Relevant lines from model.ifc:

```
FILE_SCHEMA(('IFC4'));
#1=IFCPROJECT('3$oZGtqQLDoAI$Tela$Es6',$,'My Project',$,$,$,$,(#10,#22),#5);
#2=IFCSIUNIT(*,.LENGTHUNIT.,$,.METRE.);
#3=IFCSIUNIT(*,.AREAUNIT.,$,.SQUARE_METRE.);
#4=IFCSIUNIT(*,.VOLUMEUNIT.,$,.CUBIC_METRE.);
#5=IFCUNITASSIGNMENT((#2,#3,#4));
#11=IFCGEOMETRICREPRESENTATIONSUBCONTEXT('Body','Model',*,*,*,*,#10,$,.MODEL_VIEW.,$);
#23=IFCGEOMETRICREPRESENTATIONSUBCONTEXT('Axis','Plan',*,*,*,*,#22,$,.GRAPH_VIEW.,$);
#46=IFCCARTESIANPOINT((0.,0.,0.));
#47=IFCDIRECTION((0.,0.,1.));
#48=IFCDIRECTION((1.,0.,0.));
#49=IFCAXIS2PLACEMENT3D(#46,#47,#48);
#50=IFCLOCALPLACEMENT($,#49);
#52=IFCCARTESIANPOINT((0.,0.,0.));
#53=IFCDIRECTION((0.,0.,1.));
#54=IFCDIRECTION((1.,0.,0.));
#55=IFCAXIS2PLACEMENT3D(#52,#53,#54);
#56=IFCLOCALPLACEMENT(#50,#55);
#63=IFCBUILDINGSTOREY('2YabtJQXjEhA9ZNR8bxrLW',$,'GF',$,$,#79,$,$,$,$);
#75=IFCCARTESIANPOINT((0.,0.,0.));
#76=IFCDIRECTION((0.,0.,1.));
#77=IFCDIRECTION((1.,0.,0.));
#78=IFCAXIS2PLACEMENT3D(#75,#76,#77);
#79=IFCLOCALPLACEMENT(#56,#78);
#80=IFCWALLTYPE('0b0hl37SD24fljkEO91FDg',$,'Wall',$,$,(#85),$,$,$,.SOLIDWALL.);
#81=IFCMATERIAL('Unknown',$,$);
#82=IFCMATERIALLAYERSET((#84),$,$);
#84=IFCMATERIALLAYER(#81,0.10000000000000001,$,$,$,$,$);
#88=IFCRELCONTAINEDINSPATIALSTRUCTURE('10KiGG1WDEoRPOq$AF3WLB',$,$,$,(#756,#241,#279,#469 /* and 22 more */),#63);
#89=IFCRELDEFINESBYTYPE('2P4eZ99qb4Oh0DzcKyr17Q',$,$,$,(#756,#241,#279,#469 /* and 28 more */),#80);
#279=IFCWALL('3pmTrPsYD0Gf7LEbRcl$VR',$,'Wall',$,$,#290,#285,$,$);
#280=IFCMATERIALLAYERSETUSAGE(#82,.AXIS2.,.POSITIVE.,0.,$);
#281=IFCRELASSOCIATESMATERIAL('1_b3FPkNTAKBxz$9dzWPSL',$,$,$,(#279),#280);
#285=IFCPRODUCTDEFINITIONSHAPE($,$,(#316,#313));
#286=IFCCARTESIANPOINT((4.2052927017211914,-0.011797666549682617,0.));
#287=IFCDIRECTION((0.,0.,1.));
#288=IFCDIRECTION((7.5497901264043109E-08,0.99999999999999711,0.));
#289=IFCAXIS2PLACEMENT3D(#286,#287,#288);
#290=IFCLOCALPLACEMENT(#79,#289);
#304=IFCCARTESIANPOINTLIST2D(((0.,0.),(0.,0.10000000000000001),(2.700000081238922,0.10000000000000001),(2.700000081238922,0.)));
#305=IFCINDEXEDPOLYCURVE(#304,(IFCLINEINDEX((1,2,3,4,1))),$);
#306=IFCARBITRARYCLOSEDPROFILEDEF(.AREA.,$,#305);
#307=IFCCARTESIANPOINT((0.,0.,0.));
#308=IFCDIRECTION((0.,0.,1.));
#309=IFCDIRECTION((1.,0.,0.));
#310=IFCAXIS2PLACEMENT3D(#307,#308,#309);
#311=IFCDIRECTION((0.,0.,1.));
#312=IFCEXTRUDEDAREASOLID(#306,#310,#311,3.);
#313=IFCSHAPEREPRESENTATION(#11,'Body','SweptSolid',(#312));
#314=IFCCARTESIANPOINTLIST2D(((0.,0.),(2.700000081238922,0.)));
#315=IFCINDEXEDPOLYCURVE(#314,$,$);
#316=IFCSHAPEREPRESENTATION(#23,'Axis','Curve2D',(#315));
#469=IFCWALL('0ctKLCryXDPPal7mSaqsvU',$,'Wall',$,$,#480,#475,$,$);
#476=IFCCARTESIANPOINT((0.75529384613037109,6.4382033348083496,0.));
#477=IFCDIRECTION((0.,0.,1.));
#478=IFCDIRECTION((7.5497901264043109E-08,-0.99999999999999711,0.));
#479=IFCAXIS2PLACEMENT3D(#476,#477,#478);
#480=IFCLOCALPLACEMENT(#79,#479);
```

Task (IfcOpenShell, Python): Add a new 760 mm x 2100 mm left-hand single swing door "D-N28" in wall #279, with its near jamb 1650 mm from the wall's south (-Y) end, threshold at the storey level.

```python
import numpy as np
import ifcopenshell
import ifcopenshell.api.feature
import ifcopenshell.api.geometry
import ifcopenshell.api.root
import ifcopenshell.api.spatial
import ifcopenshell.geom
import ifcopenshell.util.element
import ifcopenshell.util.placement
import ifcopenshell.util.representation
import ifcopenshell.util.shape
import ifcopenshell.util.unit

model = ifcopenshell.open("model.ifc")
unit_scale = ifcopenshell.util.unit.calculate_unit_scale(model)
settings = ifcopenshell.geom.settings()


def volume(element):
    """Net volume in cubic metres, openings subtracted."""
    shape = ifcopenshell.geom.create_shape(settings, element)
    return ifcopenshell.util.shape.get_volume(shape.geometry)


wall = model.by_guid("3pmTrPsYD0Gf7LEbRcl$VR")
storey = ifcopenshell.util.element.get_container(wall, ifc_class="IfcBuildingStorey")
context = ifcopenshell.util.representation.get_context(model, "Model", "Body", "MODEL_VIEW")
before = volume(wall)

width, height, from_end, sill = 0.76, 2.1, 1.65, 0.0  # metres

# The wall runs along its own X axis, and the end named is its -X end.
wall_shape = ifcopenshell.geom.create_shape(settings, wall)
x, y, z = ifcopenshell.util.shape.get_vertices(wall_shape.geometry).T
start = x.min() + from_end
face, thickness = float(y.min()), float(y.max() - y.min())
wall_matrix = ifcopenshell.util.placement.get_local_placement(wall.ObjectPlacement)
level = ifcopenshell.util.placement.get_local_placement(storey.ObjectPlacement)[2, 3]


def in_wall(x, y):
    """Placement at x, y metres in the wall's axes, at sill height."""
    matrix = wall_matrix.copy()
    matrix[:, 3] = wall_matrix @ np.array([x / unit_scale, y / unit_scale, 0.0, 1.0])
    matrix[2, 3] = level + sill / unit_scale
    return matrix


# Opening: a box that overshoots both wall faces by 50 mm.
opening = ifcopenshell.api.root.create_entity(model, ifc_class="IfcOpeningElement", predefined_type="OPENING")
box = ifcopenshell.api.geometry.add_wall_representation(
    model, context=context, length=width, height=height, thickness=thickness + 0.1
)
ifcopenshell.api.geometry.assign_representation(model, product=opening, representation=box)
ifcopenshell.api.geometry.edit_object_placement(model, product=opening, matrix=in_wall(start, face - 0.05), is_si=False)
ifcopenshell.api.feature.add_feature(model, feature=opening, element=wall)

door = ifcopenshell.api.root.create_entity(model, ifc_class="IfcDoor", name="D-N28", predefined_type="DOOR")
door.OverallWidth, door.OverallHeight = width / unit_scale, height / unit_scale
door.OperationType = "SINGLE_SWING_LEFT"
body = ifcopenshell.api.geometry.add_door_representation(
    model,
    context=context,
    overall_width=door.OverallWidth,
    overall_height=door.OverallHeight,
    operation_type="SINGLE_SWING_LEFT",
    lining_properties={"LiningDepth": thickness / unit_scale, "ThresholdDepth": thickness / unit_scale},
)
ifcopenshell.api.geometry.assign_representation(model, product=door, representation=body)
ifcopenshell.api.spatial.assign_container(model, products=[door], relating_structure=storey)
ifcopenshell.api.feature.add_filling(model, opening=opening, element=door)

# The lining spans the wall, so the door starts at the wall face.
ifcopenshell.api.geometry.edit_object_placement(model, product=door, matrix=in_wall(start, face), is_si=False)

after = volume(wall)

print(f"wall volume {before:.3f} -> {after:.3f} m3")

model.write("model_updated.ifc")
```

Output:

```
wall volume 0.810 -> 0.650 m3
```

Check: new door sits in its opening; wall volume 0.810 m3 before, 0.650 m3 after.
